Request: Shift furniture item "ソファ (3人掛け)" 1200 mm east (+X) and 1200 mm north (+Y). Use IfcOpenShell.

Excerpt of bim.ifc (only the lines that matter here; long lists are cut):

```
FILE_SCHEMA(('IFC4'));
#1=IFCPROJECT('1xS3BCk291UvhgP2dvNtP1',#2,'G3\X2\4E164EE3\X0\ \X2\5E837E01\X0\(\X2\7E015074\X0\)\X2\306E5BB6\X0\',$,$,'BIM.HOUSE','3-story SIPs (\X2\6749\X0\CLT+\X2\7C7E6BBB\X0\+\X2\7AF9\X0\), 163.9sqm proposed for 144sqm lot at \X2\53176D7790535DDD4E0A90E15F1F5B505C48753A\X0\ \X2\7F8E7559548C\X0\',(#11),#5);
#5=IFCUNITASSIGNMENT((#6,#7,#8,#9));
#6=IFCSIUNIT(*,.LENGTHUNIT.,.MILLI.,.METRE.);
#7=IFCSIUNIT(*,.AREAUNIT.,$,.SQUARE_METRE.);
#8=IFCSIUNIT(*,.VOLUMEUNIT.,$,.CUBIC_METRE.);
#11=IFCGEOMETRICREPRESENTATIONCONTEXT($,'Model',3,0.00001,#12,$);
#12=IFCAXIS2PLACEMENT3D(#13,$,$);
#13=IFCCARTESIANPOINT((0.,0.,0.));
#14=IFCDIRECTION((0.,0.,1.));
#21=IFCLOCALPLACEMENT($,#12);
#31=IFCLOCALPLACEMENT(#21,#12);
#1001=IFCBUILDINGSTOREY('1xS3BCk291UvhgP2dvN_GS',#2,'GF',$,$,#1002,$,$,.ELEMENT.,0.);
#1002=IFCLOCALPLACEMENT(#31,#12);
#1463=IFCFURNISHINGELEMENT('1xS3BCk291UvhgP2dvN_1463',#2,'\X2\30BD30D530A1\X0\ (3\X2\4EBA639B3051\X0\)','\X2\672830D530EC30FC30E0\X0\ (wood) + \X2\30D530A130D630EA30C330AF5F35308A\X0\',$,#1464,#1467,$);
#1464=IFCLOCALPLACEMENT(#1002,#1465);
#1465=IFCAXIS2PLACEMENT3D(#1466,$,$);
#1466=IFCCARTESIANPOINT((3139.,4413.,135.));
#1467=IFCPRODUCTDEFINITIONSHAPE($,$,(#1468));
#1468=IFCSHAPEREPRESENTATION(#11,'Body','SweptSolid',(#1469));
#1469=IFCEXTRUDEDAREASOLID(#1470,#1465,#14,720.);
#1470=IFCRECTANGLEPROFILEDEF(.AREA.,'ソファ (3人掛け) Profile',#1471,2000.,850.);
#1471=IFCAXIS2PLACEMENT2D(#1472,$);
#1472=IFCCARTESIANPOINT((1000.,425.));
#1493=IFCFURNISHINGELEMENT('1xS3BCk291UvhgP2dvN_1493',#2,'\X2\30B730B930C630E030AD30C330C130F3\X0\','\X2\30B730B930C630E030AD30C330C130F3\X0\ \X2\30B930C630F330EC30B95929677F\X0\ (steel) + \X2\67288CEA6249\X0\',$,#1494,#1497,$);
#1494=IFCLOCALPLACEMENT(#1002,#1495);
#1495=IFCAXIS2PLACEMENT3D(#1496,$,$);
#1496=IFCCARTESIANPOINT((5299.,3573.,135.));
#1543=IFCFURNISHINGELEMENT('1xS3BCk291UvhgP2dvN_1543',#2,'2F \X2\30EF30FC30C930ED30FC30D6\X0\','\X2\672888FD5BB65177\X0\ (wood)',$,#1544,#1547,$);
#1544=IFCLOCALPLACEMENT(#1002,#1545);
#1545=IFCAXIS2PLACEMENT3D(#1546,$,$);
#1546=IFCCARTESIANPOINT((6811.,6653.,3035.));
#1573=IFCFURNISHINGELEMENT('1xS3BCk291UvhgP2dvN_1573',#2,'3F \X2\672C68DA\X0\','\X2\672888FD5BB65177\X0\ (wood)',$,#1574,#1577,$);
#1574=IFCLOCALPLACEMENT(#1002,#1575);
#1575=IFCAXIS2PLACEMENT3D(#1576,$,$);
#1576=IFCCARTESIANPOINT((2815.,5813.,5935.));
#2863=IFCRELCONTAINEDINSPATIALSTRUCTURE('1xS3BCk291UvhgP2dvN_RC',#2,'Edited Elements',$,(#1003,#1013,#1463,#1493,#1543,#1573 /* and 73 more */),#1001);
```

```python
import ifcopenshell
import ifcopenshell.api.geometry
import ifcopenshell.util.placement
import ifcopenshell.util.unit

model = ifcopenshell.open("bim.ifc")
unit_scale = ifcopenshell.util.unit.calculate_unit_scale(model)

item = model.by_guid("1xS3BCk291UvhgP2dvN_1463")
matrix = ifcopenshell.util.placement.get_local_placement(item.ObjectPlacement)
matrix[0, 3] += 1.2 / unit_scale
matrix[1, 3] += 1.2 / unit_scale
ifcopenshell.api.geometry.edit_object_placement(model, product=item, matrix=matrix, is_si=False)

print(ifcopenshell.util.placement.get_local_placement(item.ObjectPlacement).round(3) + 0.0)

model.write("bim_edited.ifc")
```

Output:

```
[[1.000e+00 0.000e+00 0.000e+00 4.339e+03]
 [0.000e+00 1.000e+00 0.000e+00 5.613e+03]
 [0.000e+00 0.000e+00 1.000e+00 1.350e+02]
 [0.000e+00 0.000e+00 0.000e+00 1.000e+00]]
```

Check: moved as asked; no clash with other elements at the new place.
